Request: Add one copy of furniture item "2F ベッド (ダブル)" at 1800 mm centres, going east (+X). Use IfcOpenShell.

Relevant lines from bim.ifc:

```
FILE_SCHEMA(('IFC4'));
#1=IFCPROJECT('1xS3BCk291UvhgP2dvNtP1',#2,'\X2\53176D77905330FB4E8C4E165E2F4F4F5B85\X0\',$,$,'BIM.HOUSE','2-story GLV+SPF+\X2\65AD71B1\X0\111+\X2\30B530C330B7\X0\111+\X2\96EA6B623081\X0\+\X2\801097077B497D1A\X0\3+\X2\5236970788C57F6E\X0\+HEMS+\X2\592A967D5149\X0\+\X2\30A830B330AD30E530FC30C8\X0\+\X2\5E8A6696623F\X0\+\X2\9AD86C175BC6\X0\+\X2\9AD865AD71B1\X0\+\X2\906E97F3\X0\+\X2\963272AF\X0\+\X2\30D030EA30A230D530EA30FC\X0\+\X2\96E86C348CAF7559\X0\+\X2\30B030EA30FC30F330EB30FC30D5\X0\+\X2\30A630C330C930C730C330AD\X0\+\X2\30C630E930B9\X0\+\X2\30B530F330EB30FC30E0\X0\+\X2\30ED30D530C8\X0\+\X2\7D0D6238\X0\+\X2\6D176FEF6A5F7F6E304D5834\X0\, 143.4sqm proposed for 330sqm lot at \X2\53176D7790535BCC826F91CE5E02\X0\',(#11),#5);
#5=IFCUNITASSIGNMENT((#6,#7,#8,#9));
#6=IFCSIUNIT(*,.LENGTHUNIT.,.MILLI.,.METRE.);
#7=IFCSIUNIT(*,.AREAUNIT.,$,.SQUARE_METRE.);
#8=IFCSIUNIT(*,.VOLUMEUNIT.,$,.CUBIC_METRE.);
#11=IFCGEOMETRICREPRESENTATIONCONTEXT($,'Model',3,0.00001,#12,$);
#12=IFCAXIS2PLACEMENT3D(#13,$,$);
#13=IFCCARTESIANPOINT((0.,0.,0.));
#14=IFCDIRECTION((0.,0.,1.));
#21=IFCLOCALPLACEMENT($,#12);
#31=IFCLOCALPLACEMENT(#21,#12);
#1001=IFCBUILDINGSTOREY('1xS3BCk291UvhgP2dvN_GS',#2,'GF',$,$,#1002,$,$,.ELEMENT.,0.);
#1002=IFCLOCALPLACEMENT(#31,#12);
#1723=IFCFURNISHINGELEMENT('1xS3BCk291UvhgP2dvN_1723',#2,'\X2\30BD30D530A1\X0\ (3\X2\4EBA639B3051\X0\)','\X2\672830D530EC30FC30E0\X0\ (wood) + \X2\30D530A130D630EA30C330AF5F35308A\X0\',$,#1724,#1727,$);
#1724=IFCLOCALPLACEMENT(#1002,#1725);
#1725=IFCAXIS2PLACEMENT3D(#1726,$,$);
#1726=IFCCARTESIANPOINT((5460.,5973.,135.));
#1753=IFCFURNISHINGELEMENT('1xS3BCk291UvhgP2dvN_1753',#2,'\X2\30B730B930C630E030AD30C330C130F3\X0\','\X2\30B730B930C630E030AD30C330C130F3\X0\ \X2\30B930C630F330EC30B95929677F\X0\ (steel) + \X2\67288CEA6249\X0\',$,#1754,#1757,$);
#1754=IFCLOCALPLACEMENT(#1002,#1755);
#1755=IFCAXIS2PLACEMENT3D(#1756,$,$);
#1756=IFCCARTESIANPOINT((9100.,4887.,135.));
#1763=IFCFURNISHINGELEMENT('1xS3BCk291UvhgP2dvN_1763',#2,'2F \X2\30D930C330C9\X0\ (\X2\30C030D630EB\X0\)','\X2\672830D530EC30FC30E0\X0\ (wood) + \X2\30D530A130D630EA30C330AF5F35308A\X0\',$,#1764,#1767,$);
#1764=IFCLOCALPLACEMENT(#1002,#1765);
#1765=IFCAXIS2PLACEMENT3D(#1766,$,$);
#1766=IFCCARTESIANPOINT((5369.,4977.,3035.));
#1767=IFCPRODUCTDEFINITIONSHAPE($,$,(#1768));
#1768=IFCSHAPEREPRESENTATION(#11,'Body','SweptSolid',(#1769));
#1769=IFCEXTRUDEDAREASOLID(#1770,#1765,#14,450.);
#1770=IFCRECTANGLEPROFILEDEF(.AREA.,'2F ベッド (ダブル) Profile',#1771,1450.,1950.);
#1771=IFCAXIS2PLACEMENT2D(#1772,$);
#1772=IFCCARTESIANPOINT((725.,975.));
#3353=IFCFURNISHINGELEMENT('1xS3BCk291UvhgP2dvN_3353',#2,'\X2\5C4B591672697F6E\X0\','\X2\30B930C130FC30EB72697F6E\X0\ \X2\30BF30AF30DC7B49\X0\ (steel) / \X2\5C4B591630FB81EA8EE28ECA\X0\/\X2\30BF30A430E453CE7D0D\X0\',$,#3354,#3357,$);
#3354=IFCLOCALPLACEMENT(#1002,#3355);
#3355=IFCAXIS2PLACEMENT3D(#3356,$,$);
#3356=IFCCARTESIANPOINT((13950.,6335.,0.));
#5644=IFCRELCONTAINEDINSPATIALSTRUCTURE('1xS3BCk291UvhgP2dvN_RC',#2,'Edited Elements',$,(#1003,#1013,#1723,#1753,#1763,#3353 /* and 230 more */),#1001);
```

```python
import numpy as np
import ifcopenshell
import ifcopenshell.api.geometry
import ifcopenshell.api.root
import ifcopenshell.util.element
import ifcopenshell.util.placement
import ifcopenshell.util.unit

model = ifcopenshell.open("bim.ifc")
unit_scale = ifcopenshell.util.unit.calculate_unit_scale(model)


def reuse_history(source, copy):
    """copy_class also copies each property set's owner history, people and application; keep the originals."""
    for rel in copy.IsDefinedBy:
        if rel.is_a("IfcRelDefinesByProperties") and (history := rel.RelatingPropertyDefinition.OwnerHistory):
            rel.RelatingPropertyDefinition.OwnerHistory = source.OwnerHistory
            ifcopenshell.util.element.remove_deep2(model, history)


source = model.by_guid("1xS3BCk291UvhgP2dvN_1763")
base = ifcopenshell.util.placement.get_local_placement(source.ObjectPlacement)
step = np.array([1.0, 0.0, 0.0]) * 1.8 / unit_scale

for i in range(1, 2):
    copy = ifcopenshell.api.root.copy_class(model, product=source)
    copy.Representation = ifcopenshell.util.element.copy_deep(
        model, source.Representation, exclude=["IfcGeometricRepresentationContext", "IfcRepresentationMap"]
    )
    reuse_history(source, copy)
    matrix = base.copy()
    matrix[:3, 3] += i * step
    print("added at", matrix[:3, 3].round(3) + 0.0)
    ifcopenshell.api.geometry.edit_object_placement(model, product=copy, matrix=matrix, is_si=False)

model.write("bim_v2.ifc")
```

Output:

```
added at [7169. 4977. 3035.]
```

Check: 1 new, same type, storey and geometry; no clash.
